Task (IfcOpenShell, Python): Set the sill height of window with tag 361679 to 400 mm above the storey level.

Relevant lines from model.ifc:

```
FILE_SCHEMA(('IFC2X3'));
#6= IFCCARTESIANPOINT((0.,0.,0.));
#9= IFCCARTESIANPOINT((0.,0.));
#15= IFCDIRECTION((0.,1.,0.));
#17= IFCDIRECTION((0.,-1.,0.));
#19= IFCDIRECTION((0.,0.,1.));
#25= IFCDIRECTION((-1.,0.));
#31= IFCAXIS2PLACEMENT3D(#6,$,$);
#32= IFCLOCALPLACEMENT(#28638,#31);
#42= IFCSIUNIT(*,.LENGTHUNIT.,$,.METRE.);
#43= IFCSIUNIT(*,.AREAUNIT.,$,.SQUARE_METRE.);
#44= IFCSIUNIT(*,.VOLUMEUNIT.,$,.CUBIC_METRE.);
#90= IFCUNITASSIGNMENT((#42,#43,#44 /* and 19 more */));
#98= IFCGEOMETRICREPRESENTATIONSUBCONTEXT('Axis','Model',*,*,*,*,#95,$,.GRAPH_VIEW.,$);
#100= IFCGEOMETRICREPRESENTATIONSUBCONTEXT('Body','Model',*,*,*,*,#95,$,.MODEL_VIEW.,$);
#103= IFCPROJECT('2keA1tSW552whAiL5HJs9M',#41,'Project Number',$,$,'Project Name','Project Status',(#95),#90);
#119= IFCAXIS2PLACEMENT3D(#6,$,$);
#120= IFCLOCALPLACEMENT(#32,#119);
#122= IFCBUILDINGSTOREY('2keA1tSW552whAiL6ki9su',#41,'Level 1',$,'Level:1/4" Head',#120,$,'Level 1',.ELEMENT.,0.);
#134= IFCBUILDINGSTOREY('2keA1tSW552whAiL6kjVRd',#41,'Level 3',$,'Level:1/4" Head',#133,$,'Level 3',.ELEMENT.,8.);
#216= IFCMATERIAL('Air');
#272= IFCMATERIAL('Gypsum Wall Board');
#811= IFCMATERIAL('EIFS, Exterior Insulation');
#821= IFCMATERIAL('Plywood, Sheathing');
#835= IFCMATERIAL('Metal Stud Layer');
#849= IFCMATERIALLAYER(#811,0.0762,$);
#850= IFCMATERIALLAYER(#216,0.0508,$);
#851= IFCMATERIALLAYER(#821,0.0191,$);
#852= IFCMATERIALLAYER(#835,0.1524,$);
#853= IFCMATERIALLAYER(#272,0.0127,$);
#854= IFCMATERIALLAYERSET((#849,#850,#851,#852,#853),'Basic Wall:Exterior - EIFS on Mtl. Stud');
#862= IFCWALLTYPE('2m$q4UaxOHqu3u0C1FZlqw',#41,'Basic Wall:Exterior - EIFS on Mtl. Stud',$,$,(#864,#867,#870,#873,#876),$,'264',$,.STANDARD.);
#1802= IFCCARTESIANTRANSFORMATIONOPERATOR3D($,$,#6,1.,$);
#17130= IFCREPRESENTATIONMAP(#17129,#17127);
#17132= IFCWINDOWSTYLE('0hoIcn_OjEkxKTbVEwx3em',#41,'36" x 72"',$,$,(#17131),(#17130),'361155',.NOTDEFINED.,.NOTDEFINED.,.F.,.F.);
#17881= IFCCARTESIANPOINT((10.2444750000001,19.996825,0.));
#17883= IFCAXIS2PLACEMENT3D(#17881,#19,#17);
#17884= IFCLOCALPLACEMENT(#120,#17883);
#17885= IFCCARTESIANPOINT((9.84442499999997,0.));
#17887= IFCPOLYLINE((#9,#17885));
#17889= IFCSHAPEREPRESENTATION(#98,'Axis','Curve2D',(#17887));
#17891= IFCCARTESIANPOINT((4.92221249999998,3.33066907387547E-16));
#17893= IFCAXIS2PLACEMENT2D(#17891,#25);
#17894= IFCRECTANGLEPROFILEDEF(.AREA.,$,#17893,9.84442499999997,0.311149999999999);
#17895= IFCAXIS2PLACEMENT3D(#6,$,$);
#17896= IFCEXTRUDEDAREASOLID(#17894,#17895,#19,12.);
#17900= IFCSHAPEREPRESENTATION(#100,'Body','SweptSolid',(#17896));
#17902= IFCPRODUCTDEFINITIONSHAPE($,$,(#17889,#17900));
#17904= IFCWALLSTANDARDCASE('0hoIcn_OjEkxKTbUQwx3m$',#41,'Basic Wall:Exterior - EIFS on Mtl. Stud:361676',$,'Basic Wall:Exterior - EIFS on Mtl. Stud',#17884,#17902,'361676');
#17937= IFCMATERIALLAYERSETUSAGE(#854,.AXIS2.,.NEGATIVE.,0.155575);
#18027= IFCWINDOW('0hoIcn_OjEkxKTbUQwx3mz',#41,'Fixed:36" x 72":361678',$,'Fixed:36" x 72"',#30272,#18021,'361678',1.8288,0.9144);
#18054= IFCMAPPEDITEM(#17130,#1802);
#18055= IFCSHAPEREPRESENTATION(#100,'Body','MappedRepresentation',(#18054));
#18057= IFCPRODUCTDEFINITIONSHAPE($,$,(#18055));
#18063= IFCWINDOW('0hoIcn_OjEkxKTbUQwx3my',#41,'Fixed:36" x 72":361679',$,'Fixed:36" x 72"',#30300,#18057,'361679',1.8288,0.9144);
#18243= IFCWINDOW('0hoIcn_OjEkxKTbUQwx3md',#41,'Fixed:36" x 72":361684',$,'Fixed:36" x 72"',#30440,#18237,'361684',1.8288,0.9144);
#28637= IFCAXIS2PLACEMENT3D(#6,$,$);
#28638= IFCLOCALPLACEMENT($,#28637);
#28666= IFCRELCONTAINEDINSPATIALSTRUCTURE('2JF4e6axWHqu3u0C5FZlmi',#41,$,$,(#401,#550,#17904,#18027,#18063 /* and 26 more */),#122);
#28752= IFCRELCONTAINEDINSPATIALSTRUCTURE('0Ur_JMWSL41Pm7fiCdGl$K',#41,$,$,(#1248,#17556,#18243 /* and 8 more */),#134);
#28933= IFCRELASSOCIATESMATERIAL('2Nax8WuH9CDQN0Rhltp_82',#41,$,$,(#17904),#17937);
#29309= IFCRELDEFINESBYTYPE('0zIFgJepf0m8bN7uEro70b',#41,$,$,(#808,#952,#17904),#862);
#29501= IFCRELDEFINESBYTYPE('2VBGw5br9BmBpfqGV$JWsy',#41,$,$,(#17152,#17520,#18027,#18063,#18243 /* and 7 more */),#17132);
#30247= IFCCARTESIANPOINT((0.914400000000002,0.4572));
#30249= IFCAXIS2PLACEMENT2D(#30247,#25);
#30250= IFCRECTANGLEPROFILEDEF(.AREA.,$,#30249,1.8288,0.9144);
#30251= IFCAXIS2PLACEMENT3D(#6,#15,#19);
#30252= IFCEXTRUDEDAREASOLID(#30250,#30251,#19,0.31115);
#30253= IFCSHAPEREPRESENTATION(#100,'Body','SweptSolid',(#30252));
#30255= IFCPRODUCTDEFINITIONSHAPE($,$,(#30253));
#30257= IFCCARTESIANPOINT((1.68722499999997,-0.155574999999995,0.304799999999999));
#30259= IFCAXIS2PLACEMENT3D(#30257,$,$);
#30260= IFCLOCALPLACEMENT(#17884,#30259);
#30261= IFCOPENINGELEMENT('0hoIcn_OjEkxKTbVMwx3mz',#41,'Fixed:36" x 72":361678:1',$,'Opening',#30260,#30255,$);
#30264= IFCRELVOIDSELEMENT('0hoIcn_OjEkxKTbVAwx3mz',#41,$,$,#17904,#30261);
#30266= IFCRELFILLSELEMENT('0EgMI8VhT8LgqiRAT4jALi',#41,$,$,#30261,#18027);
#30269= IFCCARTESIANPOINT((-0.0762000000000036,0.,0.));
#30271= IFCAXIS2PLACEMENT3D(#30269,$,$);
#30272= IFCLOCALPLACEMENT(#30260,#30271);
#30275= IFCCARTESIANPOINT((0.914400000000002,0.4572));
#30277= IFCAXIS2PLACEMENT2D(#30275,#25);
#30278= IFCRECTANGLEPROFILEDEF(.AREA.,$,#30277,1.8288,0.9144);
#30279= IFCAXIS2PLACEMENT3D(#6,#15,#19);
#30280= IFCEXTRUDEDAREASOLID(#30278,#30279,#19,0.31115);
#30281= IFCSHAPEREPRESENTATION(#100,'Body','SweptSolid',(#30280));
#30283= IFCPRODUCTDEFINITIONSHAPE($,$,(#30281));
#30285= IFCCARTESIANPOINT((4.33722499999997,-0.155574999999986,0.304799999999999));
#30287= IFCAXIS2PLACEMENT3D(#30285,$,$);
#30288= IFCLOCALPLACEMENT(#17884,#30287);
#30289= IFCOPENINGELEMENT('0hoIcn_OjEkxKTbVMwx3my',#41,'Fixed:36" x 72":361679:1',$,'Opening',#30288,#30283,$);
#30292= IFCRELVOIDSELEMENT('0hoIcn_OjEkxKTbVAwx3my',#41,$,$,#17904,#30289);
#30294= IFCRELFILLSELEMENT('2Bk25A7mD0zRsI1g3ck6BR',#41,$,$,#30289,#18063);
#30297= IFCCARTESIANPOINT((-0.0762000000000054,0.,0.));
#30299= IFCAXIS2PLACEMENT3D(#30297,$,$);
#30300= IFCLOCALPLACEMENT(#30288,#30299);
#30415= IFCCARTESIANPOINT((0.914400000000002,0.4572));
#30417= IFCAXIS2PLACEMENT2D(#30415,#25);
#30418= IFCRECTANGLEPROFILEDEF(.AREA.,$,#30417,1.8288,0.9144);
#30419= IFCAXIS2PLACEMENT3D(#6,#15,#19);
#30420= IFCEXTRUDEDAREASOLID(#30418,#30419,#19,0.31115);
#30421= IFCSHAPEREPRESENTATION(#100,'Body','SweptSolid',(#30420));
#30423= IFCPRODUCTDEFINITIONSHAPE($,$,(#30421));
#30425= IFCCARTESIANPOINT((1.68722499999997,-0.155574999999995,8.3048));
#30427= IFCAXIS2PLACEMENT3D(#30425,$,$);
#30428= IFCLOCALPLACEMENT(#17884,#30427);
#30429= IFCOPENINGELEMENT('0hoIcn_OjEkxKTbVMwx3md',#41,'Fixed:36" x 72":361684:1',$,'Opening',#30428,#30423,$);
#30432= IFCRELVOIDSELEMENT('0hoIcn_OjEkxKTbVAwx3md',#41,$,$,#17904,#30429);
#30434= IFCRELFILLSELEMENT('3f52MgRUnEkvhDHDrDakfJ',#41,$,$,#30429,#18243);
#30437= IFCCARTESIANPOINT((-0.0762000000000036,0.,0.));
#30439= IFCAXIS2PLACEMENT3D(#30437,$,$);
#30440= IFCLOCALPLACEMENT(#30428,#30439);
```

```python
import numpy as np
import ifcopenshell
import ifcopenshell.api.geometry
import ifcopenshell.geom
import ifcopenshell.util.element
import ifcopenshell.util.placement
import ifcopenshell.util.shape
import ifcopenshell.util.unit

model = ifcopenshell.open("model.ifc")
unit_scale = ifcopenshell.util.unit.calculate_unit_scale(model)

window = model.by_guid("0hoIcn_OjEkxKTbUQwx3my")
opening = window.FillsVoids[0].RelatingOpeningElement
storey = ifcopenshell.util.element.get_container(window, ifc_class="IfcBuildingStorey")
level = ifcopenshell.util.placement.get_local_placement(storey.ObjectPlacement)[2, 3]

# The opening's origin need not be at the sill, so measure its lowest point.
shape = ifcopenshell.geom.create_shape(ifcopenshell.geom.settings(), opening)
bottom = ifcopenshell.util.shape.get_shape_bottom_elevation(shape, shape.geometry) / unit_scale
dz = level + 0.4 / unit_scale - bottom

shift = np.array([0.0, 0.0, dz])
# The window is placed relative to its opening, so it follows when the opening moves.
matrix = ifcopenshell.util.placement.get_local_placement(opening.ObjectPlacement)
matrix[:3, 3] += shift
ifcopenshell.api.geometry.edit_object_placement(
    model, product=opening, matrix=matrix, is_si=False, should_transform_children=True
)

print(f"moved by {dz * unit_scale:+.3f} m")

model.write("model_updated.ifc")
```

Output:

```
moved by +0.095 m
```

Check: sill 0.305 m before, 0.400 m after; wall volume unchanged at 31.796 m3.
